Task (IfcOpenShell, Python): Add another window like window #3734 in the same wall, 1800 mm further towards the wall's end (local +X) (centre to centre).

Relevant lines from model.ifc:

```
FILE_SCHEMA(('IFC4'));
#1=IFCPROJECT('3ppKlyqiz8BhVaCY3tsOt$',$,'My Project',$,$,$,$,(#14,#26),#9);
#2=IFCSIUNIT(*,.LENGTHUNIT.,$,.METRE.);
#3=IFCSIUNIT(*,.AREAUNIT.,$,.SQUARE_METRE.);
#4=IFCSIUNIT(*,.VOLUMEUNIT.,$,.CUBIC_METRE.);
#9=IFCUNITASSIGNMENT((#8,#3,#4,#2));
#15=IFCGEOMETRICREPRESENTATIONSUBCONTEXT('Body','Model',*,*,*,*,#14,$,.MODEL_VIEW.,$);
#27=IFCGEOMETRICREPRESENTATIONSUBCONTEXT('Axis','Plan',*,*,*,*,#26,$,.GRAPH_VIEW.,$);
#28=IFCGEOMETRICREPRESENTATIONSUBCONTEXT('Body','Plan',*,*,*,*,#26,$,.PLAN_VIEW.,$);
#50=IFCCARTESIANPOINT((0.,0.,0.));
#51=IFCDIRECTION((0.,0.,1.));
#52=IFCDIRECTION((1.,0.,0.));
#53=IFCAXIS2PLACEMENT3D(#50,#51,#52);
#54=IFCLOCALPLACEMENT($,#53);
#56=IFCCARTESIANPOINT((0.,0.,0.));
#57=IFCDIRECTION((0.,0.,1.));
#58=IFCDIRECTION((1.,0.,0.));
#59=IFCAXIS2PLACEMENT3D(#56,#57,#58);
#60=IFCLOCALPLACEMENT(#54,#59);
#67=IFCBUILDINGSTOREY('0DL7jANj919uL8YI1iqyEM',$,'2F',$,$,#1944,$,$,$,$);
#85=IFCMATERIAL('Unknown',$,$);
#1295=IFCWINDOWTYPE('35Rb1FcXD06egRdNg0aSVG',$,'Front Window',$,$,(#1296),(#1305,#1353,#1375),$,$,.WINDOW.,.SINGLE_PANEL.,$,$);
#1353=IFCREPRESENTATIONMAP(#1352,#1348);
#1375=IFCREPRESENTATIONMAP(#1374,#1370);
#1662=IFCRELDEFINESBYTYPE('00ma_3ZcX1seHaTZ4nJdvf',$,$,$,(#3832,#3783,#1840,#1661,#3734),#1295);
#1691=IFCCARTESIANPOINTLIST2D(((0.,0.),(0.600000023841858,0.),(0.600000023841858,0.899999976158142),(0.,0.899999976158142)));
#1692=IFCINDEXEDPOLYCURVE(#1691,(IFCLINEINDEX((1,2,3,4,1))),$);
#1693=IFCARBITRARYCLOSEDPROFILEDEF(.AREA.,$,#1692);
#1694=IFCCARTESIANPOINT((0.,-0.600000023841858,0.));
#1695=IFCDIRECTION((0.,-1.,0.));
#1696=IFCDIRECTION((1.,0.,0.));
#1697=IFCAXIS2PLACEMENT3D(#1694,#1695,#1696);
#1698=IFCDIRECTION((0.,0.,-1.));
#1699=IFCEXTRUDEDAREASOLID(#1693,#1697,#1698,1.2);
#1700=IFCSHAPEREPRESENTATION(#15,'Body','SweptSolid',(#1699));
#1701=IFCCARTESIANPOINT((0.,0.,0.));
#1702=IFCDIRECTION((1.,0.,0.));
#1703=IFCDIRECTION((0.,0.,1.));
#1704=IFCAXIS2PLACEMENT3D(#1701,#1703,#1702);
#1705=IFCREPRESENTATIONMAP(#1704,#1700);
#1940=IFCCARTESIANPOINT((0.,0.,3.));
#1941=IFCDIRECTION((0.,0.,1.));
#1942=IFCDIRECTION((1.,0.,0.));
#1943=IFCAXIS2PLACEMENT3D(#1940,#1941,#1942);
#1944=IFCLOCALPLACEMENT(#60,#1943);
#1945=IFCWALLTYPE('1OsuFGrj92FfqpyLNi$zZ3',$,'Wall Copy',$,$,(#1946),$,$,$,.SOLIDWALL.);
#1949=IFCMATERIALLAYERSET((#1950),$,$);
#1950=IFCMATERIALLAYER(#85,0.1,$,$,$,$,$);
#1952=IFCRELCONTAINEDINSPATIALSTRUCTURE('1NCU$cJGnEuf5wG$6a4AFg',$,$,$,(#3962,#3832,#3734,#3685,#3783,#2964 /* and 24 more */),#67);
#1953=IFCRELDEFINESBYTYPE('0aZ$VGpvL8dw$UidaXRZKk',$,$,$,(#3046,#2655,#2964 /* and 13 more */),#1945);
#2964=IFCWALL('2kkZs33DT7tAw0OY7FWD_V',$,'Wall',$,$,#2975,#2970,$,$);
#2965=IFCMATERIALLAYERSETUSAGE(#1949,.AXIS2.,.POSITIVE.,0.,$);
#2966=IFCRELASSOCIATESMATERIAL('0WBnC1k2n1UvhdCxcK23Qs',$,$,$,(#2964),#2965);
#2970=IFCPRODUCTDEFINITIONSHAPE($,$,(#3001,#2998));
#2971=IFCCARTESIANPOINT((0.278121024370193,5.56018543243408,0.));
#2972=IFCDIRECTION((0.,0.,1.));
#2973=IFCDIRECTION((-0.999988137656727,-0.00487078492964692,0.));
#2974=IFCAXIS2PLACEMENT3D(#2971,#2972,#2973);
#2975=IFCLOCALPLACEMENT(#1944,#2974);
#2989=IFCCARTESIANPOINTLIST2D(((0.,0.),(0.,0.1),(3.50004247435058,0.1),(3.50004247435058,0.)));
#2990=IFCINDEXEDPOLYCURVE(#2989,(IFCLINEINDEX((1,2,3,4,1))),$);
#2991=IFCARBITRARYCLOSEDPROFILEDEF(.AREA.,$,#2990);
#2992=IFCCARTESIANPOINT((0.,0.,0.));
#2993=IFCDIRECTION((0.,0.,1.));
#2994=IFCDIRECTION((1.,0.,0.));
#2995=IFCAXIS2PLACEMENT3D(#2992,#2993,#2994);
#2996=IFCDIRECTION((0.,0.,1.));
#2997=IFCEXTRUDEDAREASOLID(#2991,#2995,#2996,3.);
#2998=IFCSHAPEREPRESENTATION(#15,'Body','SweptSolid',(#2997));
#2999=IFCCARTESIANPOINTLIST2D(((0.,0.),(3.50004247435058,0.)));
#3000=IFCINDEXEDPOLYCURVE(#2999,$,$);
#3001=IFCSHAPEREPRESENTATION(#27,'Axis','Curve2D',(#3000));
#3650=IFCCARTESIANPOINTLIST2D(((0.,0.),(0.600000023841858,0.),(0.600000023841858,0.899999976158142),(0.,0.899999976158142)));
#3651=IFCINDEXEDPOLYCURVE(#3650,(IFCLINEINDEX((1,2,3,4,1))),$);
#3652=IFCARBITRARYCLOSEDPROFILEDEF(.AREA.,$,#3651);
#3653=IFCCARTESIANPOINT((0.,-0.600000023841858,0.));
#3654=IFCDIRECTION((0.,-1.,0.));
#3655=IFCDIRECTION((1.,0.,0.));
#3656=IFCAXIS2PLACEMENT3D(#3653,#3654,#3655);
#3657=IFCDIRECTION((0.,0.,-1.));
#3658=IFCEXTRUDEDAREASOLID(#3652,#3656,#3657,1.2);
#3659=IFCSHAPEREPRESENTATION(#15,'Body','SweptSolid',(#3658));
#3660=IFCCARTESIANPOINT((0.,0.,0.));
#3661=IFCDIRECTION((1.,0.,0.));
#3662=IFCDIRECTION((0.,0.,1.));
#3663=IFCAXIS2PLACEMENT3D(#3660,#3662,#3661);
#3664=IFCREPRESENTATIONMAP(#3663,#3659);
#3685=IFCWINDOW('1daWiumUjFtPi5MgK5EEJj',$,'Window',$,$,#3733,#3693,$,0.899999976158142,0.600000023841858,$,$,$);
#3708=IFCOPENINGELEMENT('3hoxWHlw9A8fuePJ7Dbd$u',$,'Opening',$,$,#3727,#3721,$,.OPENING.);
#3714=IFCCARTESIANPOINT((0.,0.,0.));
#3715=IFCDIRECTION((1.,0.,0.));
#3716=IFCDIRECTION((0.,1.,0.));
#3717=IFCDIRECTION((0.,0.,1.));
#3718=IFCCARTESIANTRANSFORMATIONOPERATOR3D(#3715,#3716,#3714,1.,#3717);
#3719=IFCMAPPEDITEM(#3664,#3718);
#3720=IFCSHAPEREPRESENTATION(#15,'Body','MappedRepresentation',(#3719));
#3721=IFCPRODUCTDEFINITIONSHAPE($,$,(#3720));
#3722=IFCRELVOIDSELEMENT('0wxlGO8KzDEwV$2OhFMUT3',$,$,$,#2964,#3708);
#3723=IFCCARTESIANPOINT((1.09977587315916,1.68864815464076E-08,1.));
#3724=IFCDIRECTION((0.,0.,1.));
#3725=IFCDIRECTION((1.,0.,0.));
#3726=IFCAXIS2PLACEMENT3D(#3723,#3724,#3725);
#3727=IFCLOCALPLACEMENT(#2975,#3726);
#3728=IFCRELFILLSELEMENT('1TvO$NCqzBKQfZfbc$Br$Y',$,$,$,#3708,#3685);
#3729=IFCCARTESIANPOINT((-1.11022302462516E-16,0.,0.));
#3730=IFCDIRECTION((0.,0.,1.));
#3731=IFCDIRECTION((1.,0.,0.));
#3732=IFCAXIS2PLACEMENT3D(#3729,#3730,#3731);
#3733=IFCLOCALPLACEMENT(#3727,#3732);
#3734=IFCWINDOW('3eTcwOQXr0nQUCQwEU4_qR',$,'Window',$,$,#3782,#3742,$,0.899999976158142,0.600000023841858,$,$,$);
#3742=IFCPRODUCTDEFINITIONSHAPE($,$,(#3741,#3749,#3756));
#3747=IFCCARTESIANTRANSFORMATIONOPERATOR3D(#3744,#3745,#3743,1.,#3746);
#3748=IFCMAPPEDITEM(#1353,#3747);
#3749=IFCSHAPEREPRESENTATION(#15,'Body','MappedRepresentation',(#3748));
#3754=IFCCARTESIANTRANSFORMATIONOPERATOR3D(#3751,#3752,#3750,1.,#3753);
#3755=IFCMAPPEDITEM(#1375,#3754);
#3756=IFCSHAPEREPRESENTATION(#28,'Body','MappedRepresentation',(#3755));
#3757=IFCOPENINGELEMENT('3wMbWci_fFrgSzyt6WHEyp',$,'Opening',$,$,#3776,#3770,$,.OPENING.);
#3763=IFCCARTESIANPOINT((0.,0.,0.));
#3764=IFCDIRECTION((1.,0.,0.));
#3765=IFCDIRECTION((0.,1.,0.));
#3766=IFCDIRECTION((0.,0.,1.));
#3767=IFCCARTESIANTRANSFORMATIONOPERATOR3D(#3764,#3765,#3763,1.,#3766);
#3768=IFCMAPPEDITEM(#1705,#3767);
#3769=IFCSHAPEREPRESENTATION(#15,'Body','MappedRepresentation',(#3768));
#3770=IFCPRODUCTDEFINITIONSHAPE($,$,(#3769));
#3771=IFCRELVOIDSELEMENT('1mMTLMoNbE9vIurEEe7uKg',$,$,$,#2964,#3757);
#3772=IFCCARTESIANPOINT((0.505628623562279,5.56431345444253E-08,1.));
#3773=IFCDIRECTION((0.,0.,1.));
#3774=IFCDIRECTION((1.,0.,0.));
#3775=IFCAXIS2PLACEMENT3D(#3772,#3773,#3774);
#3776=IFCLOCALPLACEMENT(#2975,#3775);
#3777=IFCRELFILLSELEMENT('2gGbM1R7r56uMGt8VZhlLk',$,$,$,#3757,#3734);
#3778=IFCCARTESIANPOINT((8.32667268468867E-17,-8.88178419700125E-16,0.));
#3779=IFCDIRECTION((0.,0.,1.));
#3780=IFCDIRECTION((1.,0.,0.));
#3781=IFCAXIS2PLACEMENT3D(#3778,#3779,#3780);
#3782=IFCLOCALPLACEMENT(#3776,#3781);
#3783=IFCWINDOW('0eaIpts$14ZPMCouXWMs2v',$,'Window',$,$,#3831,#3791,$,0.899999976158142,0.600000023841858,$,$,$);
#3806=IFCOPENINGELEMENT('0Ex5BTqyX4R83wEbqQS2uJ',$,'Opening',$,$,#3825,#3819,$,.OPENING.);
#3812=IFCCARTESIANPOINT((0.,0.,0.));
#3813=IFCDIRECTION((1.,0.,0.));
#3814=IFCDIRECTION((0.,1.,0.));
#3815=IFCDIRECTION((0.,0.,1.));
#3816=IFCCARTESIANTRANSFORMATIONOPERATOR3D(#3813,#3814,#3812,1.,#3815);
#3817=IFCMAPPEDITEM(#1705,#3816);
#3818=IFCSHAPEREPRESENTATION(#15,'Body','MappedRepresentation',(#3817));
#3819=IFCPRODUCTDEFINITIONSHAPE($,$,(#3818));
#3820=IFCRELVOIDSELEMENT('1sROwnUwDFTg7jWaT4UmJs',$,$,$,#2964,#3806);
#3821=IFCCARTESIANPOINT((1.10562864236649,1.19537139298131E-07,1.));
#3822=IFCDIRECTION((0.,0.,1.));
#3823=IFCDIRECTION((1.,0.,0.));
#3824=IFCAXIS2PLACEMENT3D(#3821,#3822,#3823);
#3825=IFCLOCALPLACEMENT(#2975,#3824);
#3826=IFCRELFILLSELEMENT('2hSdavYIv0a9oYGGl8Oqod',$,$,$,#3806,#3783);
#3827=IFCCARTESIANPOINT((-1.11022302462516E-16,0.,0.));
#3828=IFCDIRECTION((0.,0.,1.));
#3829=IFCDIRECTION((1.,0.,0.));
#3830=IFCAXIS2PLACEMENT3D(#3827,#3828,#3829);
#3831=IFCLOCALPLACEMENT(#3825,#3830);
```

```python
import ifcopenshell
import ifcopenshell.api.feature
import ifcopenshell.api.geometry
import ifcopenshell.api.root
import ifcopenshell.geom
import ifcopenshell.util.element
import ifcopenshell.util.placement
import ifcopenshell.util.shape
import ifcopenshell.util.unit

model = ifcopenshell.open("model.ifc")
unit_scale = ifcopenshell.util.unit.calculate_unit_scale(model)
settings = ifcopenshell.geom.settings()


def volume(element):
    """Net volume in cubic metres, openings subtracted."""
    shape = ifcopenshell.geom.create_shape(settings, element)
    return ifcopenshell.util.shape.get_volume(shape.geometry)


window = model.by_id(3734)
opening = window.FillsVoids[0].RelatingOpeningElement
wall = opening.VoidsElements[0].RelatingBuildingElement
before = volume(wall)
shift = ifcopenshell.util.placement.get_local_placement(wall.ObjectPlacement)[:3, 0] * 1.8 / unit_scale

# copy_class copies the void relationship, type, container and properties, but no geometry.
new_opening = ifcopenshell.api.root.copy_class(model, product=opening)
new_opening.Representation = ifcopenshell.util.element.copy_deep(
    model, opening.Representation, exclude=["IfcGeometricRepresentationContext", "IfcRepresentationMap"]
)
new_window = ifcopenshell.api.root.copy_class(model, product=window)
new_window.Representation = ifcopenshell.util.element.copy_deep(
    model, window.Representation, exclude=["IfcGeometricRepresentationContext", "IfcRepresentationMap"]
)
ifcopenshell.api.feature.add_filling(model, opening=new_opening, element=new_window)

for old, new in ((opening, new_opening), (window, new_window)):
    matrix = ifcopenshell.util.placement.get_local_placement(old.ObjectPlacement)
    matrix[:3, 3] += shift
    ifcopenshell.api.geometry.edit_object_placement(model, product=new, matrix=matrix, is_si=False)

after = volume(wall)

print(f"wall volume {before:.3f} -> {after:.3f} m3")

model.write("model-out.ifc")
```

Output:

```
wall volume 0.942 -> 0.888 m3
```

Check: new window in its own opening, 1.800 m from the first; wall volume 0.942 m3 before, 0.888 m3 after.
